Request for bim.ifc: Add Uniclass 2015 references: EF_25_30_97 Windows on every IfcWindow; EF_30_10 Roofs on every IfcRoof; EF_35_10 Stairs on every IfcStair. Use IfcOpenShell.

First a look at what the model holds.

```python
import ifcopenshell

model = ifcopenshell.open("bim.ifc")
print(model.schema)
print("classifications:", [c.Name for c in model.by_type("IfcClassification")])
for ifc_class in ("IfcDoor", "IfcRoof", "IfcStair", "IfcWall", "IfcWindow"):
    print(ifc_class, len(model.by_type(ifc_class)))
```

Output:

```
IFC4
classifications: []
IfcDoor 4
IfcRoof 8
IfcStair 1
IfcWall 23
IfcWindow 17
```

```python
import ifcopenshell
import ifcopenshell.api.classification

model = ifcopenshell.open("bim.ifc")

system = ifcopenshell.api.classification.add_classification(model, classification="Uniclass 2015")

codes = {
    "IfcWindow": ("EF_25_30_97", "Windows"),
    "IfcRoof": ("EF_30_10", "Roofs"),
    "IfcStair": ("EF_35_10", "Stairs"),
}
for ifc_class, (code, name) in codes.items():
    products = model.by_type(ifc_class)
    ifcopenshell.api.classification.add_reference(
        model, products=products, classification=system, identification=code, name=name
    )
    print(code, len(products))

model.write("bim_v2.ifc")
```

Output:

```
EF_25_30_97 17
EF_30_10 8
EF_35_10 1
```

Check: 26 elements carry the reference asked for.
